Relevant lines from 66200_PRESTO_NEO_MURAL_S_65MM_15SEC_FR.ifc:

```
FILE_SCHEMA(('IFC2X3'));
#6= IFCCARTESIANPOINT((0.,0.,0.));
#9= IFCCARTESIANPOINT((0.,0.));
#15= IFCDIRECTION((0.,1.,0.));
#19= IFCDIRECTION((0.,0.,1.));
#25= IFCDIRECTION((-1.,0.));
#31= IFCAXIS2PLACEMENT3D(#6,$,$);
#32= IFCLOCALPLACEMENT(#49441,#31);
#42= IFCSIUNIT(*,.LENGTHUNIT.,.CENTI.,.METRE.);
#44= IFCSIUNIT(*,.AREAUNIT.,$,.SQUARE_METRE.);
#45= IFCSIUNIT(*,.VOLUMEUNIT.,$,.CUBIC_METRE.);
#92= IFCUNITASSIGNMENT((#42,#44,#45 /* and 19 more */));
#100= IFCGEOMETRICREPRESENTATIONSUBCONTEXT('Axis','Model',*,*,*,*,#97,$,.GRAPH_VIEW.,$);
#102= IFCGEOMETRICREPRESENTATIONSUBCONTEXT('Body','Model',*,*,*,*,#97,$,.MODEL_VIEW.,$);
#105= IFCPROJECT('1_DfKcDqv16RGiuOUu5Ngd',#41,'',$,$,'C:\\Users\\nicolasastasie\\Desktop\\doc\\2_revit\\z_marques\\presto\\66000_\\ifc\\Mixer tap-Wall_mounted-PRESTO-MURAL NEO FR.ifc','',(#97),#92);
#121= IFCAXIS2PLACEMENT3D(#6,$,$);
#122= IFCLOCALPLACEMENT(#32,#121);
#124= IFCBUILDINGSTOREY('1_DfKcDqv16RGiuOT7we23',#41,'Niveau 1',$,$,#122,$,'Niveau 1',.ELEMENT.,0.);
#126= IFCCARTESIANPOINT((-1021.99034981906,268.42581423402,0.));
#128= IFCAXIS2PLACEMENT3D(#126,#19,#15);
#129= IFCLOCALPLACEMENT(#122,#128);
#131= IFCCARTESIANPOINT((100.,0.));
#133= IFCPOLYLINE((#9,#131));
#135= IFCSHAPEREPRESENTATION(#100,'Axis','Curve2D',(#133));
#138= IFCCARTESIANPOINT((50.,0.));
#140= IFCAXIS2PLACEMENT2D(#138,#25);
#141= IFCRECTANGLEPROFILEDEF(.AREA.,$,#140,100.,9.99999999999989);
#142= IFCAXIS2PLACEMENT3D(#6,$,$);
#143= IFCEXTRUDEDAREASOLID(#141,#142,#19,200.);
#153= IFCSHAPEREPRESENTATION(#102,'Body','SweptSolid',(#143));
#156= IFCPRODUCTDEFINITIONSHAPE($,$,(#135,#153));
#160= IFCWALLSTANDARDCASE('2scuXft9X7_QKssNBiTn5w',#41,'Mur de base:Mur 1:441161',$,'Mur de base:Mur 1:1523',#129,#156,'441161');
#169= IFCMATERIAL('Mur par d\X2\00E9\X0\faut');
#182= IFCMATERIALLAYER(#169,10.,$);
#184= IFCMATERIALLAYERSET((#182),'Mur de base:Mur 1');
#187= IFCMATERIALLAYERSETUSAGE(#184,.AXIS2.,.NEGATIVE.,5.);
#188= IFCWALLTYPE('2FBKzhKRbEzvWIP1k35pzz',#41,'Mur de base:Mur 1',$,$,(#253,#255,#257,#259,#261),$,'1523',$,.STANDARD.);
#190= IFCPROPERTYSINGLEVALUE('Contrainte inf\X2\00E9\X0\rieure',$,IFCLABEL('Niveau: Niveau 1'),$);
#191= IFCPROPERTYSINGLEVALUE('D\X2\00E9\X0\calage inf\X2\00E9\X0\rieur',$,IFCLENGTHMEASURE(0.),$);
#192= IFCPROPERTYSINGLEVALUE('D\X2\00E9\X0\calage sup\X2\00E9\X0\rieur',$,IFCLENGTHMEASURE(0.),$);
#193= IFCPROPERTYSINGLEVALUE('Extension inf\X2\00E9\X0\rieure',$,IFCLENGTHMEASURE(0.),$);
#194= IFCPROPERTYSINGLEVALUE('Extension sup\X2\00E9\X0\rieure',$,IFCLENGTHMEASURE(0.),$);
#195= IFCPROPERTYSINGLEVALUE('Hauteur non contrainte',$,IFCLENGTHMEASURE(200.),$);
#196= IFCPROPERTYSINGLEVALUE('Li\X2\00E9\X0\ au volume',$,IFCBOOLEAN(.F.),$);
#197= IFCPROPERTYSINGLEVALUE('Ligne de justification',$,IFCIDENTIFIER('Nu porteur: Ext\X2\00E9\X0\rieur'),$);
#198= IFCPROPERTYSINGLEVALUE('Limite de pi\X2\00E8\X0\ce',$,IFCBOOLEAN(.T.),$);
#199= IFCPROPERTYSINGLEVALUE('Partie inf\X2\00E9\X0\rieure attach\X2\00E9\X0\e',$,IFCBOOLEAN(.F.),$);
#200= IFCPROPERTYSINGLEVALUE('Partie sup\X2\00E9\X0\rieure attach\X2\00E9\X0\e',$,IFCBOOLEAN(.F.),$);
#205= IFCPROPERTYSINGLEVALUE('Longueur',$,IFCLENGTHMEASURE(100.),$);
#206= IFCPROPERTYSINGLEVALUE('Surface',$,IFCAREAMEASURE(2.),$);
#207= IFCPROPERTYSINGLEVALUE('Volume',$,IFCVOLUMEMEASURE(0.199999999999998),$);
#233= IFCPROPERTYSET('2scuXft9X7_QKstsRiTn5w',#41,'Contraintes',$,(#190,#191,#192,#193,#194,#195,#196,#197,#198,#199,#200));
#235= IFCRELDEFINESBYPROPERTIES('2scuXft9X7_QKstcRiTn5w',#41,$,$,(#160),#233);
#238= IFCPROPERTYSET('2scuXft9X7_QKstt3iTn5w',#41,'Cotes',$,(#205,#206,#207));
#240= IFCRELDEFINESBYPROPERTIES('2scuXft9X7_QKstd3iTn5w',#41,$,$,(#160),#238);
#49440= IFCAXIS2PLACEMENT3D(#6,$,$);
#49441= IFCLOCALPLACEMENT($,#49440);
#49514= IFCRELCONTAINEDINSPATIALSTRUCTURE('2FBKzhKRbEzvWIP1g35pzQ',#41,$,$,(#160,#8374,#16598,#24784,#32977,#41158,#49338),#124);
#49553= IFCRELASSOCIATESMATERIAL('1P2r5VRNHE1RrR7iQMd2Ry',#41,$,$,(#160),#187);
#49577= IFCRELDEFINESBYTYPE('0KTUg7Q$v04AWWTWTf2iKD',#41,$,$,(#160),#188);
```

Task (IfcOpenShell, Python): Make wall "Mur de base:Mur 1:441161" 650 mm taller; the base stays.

```python
import ifcopenshell
import ifcopenshell.api.pset
import ifcopenshell.geom
import ifcopenshell.util.element
import ifcopenshell.util.representation
import ifcopenshell.util.shape
import ifcopenshell.util.unit

model = ifcopenshell.open("66200_PRESTO_NEO_MURAL_S_65MM_15SEC_FR.ifc")
unit_scale = ifcopenshell.util.unit.calculate_unit_scale(model)
area_scale = ifcopenshell.util.unit.calculate_unit_scale(model, "AREAUNIT")
volume_scale = ifcopenshell.util.unit.calculate_unit_scale(model, "VOLUMEUNIT")
settings = ifcopenshell.geom.settings()


def volume(element):
    """Net volume in cubic metres, openings subtracted."""
    shape = ifcopenshell.geom.create_shape(settings, element)
    return ifcopenshell.util.shape.get_volume(shape.geometry)


wall = model.by_guid("2scuXft9X7_QKssNBiTn5w")
before = volume(wall)

body = ifcopenshell.util.representation.get_representation(wall, "Model", "Body")
solid = body.Items[0]
old_height = solid.Depth
solid.Depth += 0.65 / unit_scale
after = volume(wall)
thickness = 0.1  # wall thickness in metres

# Update the stored height, areas and volumes.
pset = model.by_id(ifcopenshell.util.element.get_pset(wall, "Contraintes", should_inherit=False)["id"])
ifcopenshell.api.pset.edit_pset(model, pset=pset, properties={
    "Hauteur non contrainte": model.create_entity("IfcLengthMeasure", solid.Depth),
})
pset = model.by_id(ifcopenshell.util.element.get_pset(wall, "Cotes", should_inherit=False)["id"])
ifcopenshell.api.pset.edit_pset(model, pset=pset, properties={
    "Surface": model.create_entity("IfcAreaMeasure", after / thickness / area_scale),
    "Volume": model.create_entity("IfcVolumeMeasure", after / volume_scale),
})

print(f"height {old_height:g} -> {solid.Depth:g}, volume {before:.3f} -> {after:.3f} m3")

model.write("66200_PRESTO_NEO_MURAL_S_65MM_15SEC_FR_edited.ifc")
```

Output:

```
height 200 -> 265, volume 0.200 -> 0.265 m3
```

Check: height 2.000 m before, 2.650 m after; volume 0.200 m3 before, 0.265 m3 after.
